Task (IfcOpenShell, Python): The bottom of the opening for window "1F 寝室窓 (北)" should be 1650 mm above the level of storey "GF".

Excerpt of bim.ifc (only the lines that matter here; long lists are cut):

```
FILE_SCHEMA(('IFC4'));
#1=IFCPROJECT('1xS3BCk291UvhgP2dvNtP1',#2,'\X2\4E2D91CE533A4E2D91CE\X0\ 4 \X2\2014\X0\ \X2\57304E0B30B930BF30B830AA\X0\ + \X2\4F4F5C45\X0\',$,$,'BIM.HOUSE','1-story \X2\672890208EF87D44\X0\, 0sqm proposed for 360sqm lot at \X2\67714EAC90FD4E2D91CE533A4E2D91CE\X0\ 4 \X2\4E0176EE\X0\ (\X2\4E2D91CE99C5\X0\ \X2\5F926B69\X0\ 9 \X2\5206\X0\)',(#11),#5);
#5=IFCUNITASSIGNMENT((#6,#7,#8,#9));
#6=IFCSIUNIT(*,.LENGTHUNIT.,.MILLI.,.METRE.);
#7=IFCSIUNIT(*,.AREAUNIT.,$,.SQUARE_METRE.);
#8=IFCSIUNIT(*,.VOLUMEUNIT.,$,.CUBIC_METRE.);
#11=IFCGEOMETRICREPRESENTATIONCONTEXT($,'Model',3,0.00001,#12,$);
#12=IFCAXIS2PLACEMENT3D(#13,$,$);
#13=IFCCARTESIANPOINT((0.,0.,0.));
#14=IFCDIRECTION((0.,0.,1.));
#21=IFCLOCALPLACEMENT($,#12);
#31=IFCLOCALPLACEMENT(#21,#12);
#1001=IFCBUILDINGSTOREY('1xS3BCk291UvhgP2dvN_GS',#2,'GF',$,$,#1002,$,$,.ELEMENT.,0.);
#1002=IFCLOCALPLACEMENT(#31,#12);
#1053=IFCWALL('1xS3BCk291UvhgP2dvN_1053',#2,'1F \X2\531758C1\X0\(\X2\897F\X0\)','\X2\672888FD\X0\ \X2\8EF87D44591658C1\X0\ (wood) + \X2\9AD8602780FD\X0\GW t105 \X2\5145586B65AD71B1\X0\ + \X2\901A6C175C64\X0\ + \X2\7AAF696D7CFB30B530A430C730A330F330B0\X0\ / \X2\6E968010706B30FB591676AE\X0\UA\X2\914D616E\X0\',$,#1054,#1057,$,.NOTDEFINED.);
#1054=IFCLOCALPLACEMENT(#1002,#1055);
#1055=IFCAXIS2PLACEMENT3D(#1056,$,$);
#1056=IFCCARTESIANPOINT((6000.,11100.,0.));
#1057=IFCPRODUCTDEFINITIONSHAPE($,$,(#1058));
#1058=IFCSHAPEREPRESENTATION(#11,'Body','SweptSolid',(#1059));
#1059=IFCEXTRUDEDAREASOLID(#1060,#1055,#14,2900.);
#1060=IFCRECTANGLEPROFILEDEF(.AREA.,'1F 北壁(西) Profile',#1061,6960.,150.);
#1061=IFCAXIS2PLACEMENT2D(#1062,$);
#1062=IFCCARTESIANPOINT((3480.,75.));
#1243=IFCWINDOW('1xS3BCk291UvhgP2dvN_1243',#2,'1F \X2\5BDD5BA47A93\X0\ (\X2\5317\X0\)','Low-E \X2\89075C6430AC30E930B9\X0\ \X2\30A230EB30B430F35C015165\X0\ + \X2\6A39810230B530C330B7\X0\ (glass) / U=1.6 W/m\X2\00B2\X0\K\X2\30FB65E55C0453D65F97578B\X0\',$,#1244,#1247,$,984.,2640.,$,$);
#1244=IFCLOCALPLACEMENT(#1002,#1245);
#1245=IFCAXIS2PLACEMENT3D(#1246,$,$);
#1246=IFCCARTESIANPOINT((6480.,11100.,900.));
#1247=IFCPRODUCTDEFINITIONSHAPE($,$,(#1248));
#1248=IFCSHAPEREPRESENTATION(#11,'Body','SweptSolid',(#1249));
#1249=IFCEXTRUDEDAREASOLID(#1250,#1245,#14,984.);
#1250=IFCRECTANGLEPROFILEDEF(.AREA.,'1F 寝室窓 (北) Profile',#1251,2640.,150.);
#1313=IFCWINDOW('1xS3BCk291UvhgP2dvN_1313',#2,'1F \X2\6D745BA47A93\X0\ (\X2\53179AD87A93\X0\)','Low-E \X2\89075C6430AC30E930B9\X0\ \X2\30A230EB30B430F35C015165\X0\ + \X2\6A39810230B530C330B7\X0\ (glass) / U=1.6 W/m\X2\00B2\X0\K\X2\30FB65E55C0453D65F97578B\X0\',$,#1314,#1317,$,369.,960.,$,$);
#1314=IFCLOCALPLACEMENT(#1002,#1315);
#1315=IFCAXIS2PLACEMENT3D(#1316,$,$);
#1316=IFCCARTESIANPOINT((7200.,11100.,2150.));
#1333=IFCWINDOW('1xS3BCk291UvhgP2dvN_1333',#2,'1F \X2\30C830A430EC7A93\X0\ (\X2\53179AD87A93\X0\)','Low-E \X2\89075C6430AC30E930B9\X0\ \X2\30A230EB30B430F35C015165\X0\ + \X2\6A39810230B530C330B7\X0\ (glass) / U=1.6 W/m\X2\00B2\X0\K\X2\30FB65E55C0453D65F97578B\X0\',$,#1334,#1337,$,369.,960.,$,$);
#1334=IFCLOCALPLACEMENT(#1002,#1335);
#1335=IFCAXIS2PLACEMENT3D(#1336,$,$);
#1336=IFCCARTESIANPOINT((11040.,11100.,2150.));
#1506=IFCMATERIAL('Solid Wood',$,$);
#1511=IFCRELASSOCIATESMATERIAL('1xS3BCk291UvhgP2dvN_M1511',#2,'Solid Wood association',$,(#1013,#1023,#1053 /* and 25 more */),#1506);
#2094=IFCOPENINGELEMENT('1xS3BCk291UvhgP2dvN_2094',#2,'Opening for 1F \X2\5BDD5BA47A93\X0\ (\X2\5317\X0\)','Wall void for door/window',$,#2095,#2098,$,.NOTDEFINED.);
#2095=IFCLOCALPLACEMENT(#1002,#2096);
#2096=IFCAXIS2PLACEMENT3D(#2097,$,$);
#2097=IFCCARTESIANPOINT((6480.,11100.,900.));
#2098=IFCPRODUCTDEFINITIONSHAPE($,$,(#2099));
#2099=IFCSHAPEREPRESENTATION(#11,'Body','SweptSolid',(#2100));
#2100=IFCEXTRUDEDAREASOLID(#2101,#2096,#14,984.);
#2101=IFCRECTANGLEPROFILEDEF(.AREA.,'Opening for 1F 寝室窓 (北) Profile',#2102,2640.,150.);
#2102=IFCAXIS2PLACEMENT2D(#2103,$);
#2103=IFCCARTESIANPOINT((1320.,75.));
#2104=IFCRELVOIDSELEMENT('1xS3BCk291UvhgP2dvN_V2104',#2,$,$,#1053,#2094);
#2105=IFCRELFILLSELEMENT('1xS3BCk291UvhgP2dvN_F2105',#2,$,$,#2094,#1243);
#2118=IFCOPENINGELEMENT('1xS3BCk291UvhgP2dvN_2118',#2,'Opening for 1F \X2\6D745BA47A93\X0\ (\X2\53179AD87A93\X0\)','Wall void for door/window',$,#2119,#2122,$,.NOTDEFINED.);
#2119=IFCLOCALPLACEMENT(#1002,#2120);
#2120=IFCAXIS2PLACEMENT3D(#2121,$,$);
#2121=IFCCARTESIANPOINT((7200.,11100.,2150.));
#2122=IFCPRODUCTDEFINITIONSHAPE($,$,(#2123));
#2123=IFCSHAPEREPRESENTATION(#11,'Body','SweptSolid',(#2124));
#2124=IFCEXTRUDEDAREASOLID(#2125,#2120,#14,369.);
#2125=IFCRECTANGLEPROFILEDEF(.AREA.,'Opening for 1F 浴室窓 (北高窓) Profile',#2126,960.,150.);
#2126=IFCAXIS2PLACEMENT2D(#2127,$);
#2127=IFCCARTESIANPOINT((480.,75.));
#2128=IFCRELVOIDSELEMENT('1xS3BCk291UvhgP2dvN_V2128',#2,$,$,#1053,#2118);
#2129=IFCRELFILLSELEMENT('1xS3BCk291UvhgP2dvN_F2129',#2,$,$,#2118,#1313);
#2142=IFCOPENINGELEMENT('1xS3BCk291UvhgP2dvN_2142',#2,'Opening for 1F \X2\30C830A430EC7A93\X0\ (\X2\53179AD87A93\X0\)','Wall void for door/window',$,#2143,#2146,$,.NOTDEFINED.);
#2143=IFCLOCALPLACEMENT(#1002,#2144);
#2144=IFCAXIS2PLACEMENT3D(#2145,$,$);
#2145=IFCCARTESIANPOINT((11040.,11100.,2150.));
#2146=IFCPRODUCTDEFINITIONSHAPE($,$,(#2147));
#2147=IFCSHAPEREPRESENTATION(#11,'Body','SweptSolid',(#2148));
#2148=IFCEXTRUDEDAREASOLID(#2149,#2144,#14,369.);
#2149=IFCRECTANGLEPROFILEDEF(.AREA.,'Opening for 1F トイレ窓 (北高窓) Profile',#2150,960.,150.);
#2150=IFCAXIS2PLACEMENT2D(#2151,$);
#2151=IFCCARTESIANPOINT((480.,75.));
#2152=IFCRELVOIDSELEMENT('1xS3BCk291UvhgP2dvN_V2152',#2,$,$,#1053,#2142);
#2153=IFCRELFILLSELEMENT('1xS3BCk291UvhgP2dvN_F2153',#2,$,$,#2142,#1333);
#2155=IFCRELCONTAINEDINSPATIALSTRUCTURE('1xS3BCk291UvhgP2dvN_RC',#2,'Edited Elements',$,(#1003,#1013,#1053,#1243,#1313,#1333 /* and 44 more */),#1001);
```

```python
import numpy as np
import ifcopenshell
import ifcopenshell.api.geometry
import ifcopenshell.geom
import ifcopenshell.util.element
import ifcopenshell.util.placement
import ifcopenshell.util.shape
import ifcopenshell.util.unit

model = ifcopenshell.open("bim.ifc")
unit_scale = ifcopenshell.util.unit.calculate_unit_scale(model)

window = model.by_id(1243)
opening = window.FillsVoids[0].RelatingOpeningElement
storey = ifcopenshell.util.element.get_container(window, ifc_class="IfcBuildingStorey")
level = ifcopenshell.util.placement.get_local_placement(storey.ObjectPlacement)[2, 3]

# The opening's origin need not be at the sill, so measure its lowest point.
shape = ifcopenshell.geom.create_shape(ifcopenshell.geom.settings(), opening)
bottom = ifcopenshell.util.shape.get_shape_bottom_elevation(shape, shape.geometry) / unit_scale
dz = level + 1.65 / unit_scale - bottom

shift = np.array([0.0, 0.0, dz])
# The window is not placed relative to its opening, so move both.
for product in (opening, window):
    matrix = ifcopenshell.util.placement.get_local_placement(product.ObjectPlacement)
    matrix[:3, 3] += shift
    ifcopenshell.api.geometry.edit_object_placement(model, product=product, matrix=matrix, is_si=False)

print(f"moved by {dz * unit_scale:+.3f} m")

model.write("bim_edited.ifc")
```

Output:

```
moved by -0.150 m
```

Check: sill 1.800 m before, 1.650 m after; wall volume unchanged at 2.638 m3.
